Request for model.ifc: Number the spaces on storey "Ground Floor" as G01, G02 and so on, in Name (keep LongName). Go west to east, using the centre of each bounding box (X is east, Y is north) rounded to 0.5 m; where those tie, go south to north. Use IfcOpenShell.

First a look at what the model holds.

```python
import ifcopenshell
import ifcopenshell.util.element
import ifcopenshell.util.placement

model = ifcopenshell.open("model.ifc")
print(model.schema)
storey = next(s for s in model.by_type("IfcBuildingStorey") if s.Name == "Ground Floor")
spaces = [e for e in ifcopenshell.util.element.get_decomposition(storey) if e.is_a("IfcSpace")]
for e in sorted(spaces, key=lambda e: e.id()):
    origin = ifcopenshell.util.placement.get_local_placement(e.ObjectPlacement)[:3, 3]
    print(e.id(), e.Name, e.LongName, origin.round(2) + 0.0, sep=" | ")
```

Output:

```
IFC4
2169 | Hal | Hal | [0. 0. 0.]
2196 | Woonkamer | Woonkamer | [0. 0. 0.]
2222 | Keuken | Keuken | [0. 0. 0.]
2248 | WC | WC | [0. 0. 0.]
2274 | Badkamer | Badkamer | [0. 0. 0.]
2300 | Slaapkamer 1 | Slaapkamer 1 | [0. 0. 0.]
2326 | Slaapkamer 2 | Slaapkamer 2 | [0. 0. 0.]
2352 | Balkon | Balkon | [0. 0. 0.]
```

```python
import ifcopenshell
import ifcopenshell.geom
import ifcopenshell.util.element
import ifcopenshell.util.shape

model = ifcopenshell.open("model.ifc")
settings = ifcopenshell.geom.settings()
settings.set("use-world-coords", True)


def centre(element):
    shape = ifcopenshell.geom.create_shape(settings, element)
    return ifcopenshell.util.shape.get_bbox_centroid(shape.geometry)


storey = next(s for s in model.by_type("IfcBuildingStorey") if s.Name == "Ground Floor")
spaces = [e for e in ifcopenshell.util.element.get_decomposition(storey) if e.is_a("IfcSpace")]

# Insertion points can sit at a corner or the storey origin, so sort by the geometry (in metres).
centres = {e: centre(e) for e in spaces}
spaces.sort(key=lambda e: (round(centres[e][0] / 0.5), centres[e][1]))

for i, e in enumerate(spaces, start=1):
    number = f"G{i:02d}"
    e.Name = number
    print(e.id(), number)

model.write("model-out.ifc")
```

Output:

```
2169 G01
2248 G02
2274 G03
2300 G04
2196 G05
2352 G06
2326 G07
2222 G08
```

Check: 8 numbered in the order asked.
